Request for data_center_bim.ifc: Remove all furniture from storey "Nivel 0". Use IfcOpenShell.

First a look at what the model holds.

```python
import ifcopenshell
import ifcopenshell.util.element

model = ifcopenshell.open("data_center_bim.ifc")
print(model.schema)
storey = next(s for s in model.by_type("IfcBuildingStorey") if s.Name == "Nivel 0")
furniture = [e for e in ifcopenshell.util.element.get_decomposition(storey) if e.is_a("IfcFurnishingElement")]
seen = {}
for e in furniture:
    element_type = ifcopenshell.util.element.get_type(e)
    name = element_type.Name if element_type not in (None, e) else None
    seen[name] = seen.get(name, 0) + 1
for name, count in sorted(seen.items(), key=str):
    print(count, "x", name)
```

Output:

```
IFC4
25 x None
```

```python
import ifcopenshell
import ifcopenshell.api.root
import ifcopenshell.util.element

model = ifcopenshell.open("data_center_bim.ifc")

storey = next(s for s in model.by_type("IfcBuildingStorey") if s.Name == "Nivel 0")
furniture = [e for e in ifcopenshell.util.element.get_decomposition(storey) if e.is_a("IfcFurnishingElement")]

for e in furniture:
    ifcopenshell.api.root.remove_product(model, product=e)
print(len(furniture), "removed")

model.write("data_center_bim_edited.ifc")
```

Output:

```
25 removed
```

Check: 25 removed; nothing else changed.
